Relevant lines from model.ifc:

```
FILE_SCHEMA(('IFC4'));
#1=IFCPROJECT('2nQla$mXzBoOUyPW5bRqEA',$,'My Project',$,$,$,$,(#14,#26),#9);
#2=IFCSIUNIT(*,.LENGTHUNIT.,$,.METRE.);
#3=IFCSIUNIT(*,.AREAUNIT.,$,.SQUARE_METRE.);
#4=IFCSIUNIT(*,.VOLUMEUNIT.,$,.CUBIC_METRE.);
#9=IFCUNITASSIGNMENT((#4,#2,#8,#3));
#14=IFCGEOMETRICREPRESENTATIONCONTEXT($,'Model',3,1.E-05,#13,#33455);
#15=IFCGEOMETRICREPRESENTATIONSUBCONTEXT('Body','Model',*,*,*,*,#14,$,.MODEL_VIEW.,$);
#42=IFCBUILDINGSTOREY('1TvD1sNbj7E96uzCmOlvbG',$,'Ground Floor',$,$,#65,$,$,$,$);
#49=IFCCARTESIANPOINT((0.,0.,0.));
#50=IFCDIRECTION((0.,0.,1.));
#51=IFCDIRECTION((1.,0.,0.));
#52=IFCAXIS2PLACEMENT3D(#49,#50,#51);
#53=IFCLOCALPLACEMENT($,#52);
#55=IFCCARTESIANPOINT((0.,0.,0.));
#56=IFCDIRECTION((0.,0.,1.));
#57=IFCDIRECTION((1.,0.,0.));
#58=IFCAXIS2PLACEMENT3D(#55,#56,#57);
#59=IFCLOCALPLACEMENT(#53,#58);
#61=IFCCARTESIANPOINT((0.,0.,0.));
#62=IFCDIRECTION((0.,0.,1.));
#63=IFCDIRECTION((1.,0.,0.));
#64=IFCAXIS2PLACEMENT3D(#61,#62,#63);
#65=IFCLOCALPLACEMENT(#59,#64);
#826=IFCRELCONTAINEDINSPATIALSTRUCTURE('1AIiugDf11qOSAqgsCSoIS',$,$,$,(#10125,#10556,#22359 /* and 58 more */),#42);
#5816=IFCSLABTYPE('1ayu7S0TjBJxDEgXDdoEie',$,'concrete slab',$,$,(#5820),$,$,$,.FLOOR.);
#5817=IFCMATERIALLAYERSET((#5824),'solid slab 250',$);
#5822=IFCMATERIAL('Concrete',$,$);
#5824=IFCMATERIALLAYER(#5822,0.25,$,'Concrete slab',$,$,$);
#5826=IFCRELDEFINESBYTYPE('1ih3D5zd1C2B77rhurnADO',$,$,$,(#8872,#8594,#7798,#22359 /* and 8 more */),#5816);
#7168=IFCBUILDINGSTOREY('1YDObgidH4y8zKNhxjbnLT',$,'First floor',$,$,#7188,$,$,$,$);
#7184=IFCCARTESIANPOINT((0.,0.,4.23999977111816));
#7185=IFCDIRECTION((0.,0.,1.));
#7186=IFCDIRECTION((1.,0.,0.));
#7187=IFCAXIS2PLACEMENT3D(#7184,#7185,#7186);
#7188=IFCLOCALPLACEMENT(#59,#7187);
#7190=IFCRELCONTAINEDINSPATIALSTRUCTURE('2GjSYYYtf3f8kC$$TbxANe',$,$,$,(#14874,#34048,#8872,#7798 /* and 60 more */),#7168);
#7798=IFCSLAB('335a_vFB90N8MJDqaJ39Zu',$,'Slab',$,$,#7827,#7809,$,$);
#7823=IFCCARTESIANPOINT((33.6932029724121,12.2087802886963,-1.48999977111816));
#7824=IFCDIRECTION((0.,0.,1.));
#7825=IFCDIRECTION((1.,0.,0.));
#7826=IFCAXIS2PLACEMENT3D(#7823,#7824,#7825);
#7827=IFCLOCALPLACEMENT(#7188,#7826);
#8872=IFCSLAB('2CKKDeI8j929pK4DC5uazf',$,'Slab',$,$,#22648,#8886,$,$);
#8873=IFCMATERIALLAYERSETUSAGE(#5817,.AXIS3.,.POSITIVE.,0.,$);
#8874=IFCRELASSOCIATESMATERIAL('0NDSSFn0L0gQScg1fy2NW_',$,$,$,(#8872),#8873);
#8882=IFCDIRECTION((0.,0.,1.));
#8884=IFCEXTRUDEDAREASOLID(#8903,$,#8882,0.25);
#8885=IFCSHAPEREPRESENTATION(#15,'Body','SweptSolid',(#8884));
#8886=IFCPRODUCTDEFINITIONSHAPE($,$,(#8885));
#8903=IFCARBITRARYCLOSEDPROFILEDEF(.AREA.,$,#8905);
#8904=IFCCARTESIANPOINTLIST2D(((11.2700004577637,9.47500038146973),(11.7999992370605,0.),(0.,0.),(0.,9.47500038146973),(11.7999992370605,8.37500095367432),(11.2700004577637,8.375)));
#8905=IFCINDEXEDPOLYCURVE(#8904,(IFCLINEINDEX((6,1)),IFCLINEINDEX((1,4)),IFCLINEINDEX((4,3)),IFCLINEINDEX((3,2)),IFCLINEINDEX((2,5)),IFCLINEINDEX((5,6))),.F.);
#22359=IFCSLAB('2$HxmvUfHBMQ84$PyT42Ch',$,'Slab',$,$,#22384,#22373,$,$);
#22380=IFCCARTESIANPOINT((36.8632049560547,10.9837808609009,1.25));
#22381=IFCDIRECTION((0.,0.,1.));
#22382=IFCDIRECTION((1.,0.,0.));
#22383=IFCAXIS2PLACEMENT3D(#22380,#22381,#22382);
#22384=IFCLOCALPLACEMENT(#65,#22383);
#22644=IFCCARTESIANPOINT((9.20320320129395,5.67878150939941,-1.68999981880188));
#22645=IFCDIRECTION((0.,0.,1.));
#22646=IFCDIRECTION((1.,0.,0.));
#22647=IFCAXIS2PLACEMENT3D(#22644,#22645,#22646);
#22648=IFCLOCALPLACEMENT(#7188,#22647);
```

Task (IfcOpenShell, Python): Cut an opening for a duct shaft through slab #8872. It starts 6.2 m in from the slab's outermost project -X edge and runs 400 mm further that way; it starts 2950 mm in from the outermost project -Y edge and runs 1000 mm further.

```python
import numpy as np
import ifcopenshell
import ifcopenshell.api.feature
import ifcopenshell.api.geometry
import ifcopenshell.api.root
import ifcopenshell.geom
import ifcopenshell.util.placement
import ifcopenshell.util.representation
import ifcopenshell.util.shape
import ifcopenshell.util.unit

model = ifcopenshell.open("model.ifc")
unit_scale = ifcopenshell.util.unit.calculate_unit_scale(model)
settings = ifcopenshell.geom.settings()


def volume(element):
    """Net volume in cubic metres, openings subtracted."""
    shape = ifcopenshell.geom.create_shape(settings, element)
    return ifcopenshell.util.shape.get_volume(shape.geometry)


slab = model.by_guid("2CKKDeI8j929pK4DC5uazf")
before = volume(slab)

# Extent in the slab's own axes, in metres. The edges named are its -X and -Y sides.
slab_shape = ifcopenshell.geom.create_shape(settings, slab)
vertices = ifcopenshell.util.shape.get_vertices(slab_shape.geometry)
x_min, y_min, bottom = vertices.min(axis=0)
top = vertices[:, 2].max()

opening = ifcopenshell.api.root.create_entity(model, ifc_class="IfcOpeningElement", name="Duct shaft opening", predefined_type="OPENING")
context = ifcopenshell.util.representation.get_context(model, "Model", "Body", "MODEL_VIEW")
width, depth = 0.4, 1
outline = [(0.0, 0.0), (width, 0.0), (width, depth), (0.0, depth), (0.0, 0.0)]
# Overshoot both faces by 50 mm so the cut is clean.
shape = ifcopenshell.api.geometry.add_slab_representation(
    model, context=context, depth=top - bottom + 0.1, polyline=outline
)
ifcopenshell.api.geometry.assign_representation(model, product=opening, representation=shape)

matrix = ifcopenshell.util.placement.get_local_placement(slab.ObjectPlacement)
matrix[:, 3] = matrix @ np.append(np.array([x_min + 6.2, y_min + 2.95, bottom - 0.05]) / unit_scale, 1.0)
ifcopenshell.api.geometry.edit_object_placement(model, product=opening, matrix=matrix, is_si=False)
ifcopenshell.api.feature.add_feature(model, feature=opening, element=slab)

after = volume(slab)

print(f"slab volume {before:.3f} -> {after:.3f} m3")

model.write("model-out.ifc")
```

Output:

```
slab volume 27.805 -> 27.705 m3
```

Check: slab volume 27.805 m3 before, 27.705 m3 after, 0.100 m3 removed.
